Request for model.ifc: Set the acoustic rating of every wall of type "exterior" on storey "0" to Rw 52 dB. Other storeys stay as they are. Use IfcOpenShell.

First a look at what the model holds.

```python
import ifcopenshell
import ifcopenshell.util.element

model = ifcopenshell.open("model.ifc")
print(model.schema)
storey = next(s for s in model.by_type("IfcBuildingStorey") if s.Name == "0")
walls = [e for e in ifcopenshell.util.element.get_decomposition(storey) if e.is_a("IfcWall")]
seen = {}
for e in walls:
    element_type = ifcopenshell.util.element.get_type(e)
    key = (element_type.Name if element_type != e and element_type else None, ifcopenshell.util.element.get_pset(e, "Pset_WallCommon", "AcousticRating"))
    seen[key] = seen.get(key, 0) + 1
for (name, value), count in sorted(seen.items(), key=str):
    print(count, "x", name, "|", value)
```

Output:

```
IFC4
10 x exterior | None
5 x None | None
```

```python
import ifcopenshell
import ifcopenshell.api.pset
import ifcopenshell.util.element

model = ifcopenshell.open("model.ifc")

storey = next(s for s in model.by_type("IfcBuildingStorey") if s.Name == "0")
walls = [e for e in ifcopenshell.util.element.get_decomposition(storey) if e.is_a("IfcWall")]

count = 0
for e in walls:
    element_type = ifcopenshell.util.element.get_type(e)
    if element_type in (None, e) or element_type.Name != "exterior":
        continue
    # add_pset returns the element's existing set when there is one.
    pset = ifcopenshell.api.pset.add_pset(model, product=e, name="Pset_WallCommon")
    ifcopenshell.api.pset.edit_pset(model, pset=pset, properties={"AcousticRating": "Rw 52 dB"})
    count += 1

print(count, "walls updated")

model.write("model_v2.ifc")
```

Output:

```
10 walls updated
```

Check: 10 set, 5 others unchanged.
